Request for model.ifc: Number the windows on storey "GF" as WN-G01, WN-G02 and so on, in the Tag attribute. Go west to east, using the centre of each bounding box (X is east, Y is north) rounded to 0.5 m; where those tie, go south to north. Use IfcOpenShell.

First a look at what the model holds.

```python
import ifcopenshell
import ifcopenshell.util.element
import ifcopenshell.util.placement

model = ifcopenshell.open("model.ifc")
print(model.schema)
storey = next(s for s in model.by_type("IfcBuildingStorey") if s.Name == "GF")
windows = [e for e in ifcopenshell.util.element.get_decomposition(storey) if e.is_a("IfcWindow")]
for e in sorted(windows, key=lambda e: e.id()):
    origin = ifcopenshell.util.placement.get_local_placement(e.ObjectPlacement)[:3, 3]
    print(e.id(), e.Tag, e.Name, origin.round(2) + 0.0, sep=" | ")
```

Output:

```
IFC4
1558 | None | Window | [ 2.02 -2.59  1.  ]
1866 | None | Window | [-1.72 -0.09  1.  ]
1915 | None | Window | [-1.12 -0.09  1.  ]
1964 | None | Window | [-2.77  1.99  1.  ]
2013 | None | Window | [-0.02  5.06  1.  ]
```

```python
import ifcopenshell
import ifcopenshell.geom
import ifcopenshell.util.element
import ifcopenshell.util.shape

model = ifcopenshell.open("model.ifc")
settings = ifcopenshell.geom.settings()
settings.set("use-world-coords", True)


def centre(element):
    shape = ifcopenshell.geom.create_shape(settings, element)
    return ifcopenshell.util.shape.get_bbox_centroid(shape.geometry)


storey = next(s for s in model.by_type("IfcBuildingStorey") if s.Name == "GF")
windows = [e for e in ifcopenshell.util.element.get_decomposition(storey) if e.is_a("IfcWindow")]

# Insertion points can sit at a corner or the storey origin, so sort by the geometry (in metres).
centres = {e: centre(e) for e in windows}
windows.sort(key=lambda e: (round(centres[e][0] / 0.5), centres[e][1]))

for i, e in enumerate(windows, start=1):
    number = f"WN-G{i:02d}"
    e.Tag = number
    print(e.id(), number)

model.write("model_v2.ifc")
```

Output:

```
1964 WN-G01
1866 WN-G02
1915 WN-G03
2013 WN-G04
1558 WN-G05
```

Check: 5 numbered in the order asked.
